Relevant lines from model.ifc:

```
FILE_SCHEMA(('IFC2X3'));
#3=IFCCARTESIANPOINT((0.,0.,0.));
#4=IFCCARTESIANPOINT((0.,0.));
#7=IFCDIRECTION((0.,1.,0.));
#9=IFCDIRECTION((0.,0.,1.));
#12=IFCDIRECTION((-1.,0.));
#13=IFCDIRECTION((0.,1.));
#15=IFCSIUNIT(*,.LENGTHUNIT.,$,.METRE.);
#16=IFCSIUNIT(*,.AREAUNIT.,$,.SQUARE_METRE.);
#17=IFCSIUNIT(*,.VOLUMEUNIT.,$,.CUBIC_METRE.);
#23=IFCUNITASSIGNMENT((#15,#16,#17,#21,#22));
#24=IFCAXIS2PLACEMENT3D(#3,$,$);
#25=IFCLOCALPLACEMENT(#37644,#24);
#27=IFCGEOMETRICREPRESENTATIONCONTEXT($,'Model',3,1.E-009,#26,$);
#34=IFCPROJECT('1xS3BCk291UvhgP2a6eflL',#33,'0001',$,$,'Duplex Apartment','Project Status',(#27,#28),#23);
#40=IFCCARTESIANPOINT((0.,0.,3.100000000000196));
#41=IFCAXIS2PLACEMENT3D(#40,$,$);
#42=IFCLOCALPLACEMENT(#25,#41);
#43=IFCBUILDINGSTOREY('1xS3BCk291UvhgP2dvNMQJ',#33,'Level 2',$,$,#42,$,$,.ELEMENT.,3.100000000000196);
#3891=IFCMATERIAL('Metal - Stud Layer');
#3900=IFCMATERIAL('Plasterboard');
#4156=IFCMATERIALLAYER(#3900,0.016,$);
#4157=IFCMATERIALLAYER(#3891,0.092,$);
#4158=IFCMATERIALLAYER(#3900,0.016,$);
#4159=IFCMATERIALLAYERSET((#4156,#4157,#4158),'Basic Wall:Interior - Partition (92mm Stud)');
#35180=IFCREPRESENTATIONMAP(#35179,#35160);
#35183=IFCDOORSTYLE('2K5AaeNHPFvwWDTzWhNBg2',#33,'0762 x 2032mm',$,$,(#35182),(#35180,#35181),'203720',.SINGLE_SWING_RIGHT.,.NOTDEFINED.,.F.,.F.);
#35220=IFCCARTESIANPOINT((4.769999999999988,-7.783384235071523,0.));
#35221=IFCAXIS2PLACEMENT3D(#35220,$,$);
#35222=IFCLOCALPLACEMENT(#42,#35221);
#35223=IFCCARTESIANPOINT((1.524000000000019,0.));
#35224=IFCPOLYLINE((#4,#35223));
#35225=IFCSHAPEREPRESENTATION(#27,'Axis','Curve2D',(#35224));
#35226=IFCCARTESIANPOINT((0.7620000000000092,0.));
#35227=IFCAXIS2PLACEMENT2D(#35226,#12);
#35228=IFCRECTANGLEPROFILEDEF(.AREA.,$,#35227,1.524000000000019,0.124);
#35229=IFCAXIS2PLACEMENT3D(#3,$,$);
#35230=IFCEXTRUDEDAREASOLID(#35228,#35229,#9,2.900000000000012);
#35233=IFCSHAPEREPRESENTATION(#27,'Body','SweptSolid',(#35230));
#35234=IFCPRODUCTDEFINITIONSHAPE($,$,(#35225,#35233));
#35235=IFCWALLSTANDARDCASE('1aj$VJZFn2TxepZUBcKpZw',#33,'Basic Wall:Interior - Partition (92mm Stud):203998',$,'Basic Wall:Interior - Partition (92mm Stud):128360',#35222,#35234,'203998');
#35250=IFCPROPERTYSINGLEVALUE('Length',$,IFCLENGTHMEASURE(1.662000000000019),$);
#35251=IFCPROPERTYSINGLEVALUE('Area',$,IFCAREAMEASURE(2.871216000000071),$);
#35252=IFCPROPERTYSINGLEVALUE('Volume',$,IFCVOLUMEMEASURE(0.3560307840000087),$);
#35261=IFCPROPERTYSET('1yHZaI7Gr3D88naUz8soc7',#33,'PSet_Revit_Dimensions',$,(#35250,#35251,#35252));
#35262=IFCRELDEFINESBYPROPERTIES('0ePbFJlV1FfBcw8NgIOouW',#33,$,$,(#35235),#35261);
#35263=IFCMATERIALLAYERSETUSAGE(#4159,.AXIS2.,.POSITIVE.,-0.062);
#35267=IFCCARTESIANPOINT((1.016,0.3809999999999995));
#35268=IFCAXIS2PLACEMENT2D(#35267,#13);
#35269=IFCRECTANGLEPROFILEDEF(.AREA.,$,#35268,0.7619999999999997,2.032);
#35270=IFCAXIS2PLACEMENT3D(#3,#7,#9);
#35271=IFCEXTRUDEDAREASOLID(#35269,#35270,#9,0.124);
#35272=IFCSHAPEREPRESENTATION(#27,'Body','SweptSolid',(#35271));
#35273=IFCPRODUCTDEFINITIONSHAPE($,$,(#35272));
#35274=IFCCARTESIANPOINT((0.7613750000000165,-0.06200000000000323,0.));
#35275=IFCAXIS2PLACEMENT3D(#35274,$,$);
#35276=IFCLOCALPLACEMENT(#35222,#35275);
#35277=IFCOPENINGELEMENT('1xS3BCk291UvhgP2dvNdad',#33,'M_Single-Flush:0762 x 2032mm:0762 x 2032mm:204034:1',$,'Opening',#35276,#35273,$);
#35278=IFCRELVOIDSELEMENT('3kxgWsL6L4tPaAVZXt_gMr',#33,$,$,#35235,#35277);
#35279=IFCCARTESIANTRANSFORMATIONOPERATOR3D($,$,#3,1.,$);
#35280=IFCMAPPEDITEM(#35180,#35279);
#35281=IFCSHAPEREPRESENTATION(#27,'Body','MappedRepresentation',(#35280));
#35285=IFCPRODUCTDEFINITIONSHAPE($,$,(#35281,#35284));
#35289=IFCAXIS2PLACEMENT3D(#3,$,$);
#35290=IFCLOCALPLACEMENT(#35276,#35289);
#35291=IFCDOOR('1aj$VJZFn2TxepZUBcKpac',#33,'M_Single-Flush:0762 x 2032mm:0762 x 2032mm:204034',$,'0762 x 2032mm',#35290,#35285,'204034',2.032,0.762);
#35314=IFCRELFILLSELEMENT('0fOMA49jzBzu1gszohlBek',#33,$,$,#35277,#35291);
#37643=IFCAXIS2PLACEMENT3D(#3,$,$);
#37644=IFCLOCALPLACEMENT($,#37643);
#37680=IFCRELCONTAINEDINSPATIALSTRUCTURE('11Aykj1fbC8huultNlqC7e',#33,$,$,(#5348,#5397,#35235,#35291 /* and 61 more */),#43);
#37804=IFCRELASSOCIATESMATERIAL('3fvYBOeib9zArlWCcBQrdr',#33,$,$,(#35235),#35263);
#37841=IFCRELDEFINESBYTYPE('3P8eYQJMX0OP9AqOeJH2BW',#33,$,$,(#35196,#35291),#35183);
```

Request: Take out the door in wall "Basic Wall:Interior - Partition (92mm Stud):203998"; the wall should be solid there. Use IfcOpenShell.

```python
import ifcopenshell
import ifcopenshell.api.feature
import ifcopenshell.api.pset
import ifcopenshell.api.root
import ifcopenshell.geom
import ifcopenshell.util.element
import ifcopenshell.util.shape
import ifcopenshell.util.unit

model = ifcopenshell.open("model.ifc")
area_scale = ifcopenshell.util.unit.calculate_unit_scale(model, "AREAUNIT")
volume_scale = ifcopenshell.util.unit.calculate_unit_scale(model, "VOLUMEUNIT")
settings = ifcopenshell.geom.settings()


def volume(element):
    """Net volume in cubic metres, openings subtracted."""
    shape = ifcopenshell.geom.create_shape(settings, element)
    return ifcopenshell.util.shape.get_volume(shape.geometry)


door = model.by_guid("1aj$VJZFn2TxepZUBcKpac")
opening = door.FillsVoids[0].RelatingOpeningElement
wall = opening.VoidsElements[0].RelatingBuildingElement
before = volume(wall)

ifcopenshell.api.root.remove_product(model, product=door)
ifcopenshell.api.feature.remove_feature(model, feature=opening)

after = volume(wall)
thickness = 0.124  # wall thickness in metres

# Update the wall's stored quantities.
pset = model.by_id(ifcopenshell.util.element.get_pset(wall, "PSet_Revit_Dimensions", should_inherit=False)["id"])
ifcopenshell.api.pset.edit_pset(model, pset=pset, properties={
    "Area": model.create_entity("IfcAreaMeasure", after / thickness / area_scale),
    "Volume": model.create_entity("IfcVolumeMeasure", after / volume_scale),
})

print(f"wall volume {before:.3f} -> {after:.3f} m3")

model.write("model_v2.ifc")
```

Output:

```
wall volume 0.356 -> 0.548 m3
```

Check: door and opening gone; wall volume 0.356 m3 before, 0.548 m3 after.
